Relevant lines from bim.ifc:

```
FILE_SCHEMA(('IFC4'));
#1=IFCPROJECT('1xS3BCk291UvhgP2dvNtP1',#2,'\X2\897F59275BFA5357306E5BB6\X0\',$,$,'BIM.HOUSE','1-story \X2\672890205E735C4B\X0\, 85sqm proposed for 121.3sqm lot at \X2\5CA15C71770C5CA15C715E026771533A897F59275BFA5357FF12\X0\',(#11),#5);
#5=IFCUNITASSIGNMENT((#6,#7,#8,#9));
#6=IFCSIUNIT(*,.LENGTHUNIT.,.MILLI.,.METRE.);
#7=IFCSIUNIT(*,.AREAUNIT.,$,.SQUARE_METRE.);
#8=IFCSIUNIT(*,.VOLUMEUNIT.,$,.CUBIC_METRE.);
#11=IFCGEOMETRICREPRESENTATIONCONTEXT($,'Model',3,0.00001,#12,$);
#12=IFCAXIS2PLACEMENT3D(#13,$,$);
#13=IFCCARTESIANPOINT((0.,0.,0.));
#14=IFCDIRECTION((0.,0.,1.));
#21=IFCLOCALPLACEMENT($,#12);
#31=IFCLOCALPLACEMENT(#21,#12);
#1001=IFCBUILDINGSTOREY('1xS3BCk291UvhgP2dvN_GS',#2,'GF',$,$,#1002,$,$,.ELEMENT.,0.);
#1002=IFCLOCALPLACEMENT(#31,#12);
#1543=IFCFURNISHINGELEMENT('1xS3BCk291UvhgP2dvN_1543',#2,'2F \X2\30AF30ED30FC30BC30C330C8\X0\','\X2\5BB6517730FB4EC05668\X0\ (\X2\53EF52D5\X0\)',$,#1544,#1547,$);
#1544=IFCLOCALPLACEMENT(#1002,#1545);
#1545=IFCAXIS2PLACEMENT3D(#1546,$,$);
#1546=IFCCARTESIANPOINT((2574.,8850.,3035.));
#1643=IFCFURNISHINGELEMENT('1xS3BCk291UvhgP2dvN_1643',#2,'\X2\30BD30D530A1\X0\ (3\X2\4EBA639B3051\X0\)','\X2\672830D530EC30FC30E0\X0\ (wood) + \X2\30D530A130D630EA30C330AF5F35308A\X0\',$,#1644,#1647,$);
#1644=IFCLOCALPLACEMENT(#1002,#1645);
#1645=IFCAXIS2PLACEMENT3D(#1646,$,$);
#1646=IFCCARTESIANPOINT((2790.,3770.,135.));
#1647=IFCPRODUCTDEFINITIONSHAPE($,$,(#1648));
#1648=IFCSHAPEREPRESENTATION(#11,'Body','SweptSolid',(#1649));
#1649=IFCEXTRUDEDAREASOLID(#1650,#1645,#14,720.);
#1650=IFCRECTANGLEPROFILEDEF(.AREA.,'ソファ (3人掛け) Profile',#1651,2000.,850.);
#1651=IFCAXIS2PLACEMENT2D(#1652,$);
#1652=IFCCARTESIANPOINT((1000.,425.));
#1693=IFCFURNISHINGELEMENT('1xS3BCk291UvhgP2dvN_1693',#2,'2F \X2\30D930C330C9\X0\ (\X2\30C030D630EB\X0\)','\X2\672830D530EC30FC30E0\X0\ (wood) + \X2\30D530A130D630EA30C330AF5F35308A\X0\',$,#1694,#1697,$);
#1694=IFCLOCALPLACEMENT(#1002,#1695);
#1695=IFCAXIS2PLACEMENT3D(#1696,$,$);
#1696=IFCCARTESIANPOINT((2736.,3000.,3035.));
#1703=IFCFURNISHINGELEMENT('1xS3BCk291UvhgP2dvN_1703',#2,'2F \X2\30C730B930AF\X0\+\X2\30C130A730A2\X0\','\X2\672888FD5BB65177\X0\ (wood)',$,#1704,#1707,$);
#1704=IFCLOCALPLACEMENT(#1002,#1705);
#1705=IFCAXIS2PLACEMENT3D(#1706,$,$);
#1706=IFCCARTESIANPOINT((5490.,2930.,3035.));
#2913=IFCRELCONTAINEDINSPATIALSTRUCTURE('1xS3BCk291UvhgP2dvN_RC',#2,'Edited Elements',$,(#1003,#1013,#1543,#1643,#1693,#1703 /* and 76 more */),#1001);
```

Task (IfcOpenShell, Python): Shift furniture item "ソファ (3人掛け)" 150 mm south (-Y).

```python
import ifcopenshell
import ifcopenshell.api.geometry
import ifcopenshell.util.placement
import ifcopenshell.util.unit

model = ifcopenshell.open("bim.ifc")
unit_scale = ifcopenshell.util.unit.calculate_unit_scale(model)

item = model.by_guid("1xS3BCk291UvhgP2dvN_1643")
matrix = ifcopenshell.util.placement.get_local_placement(item.ObjectPlacement)
matrix[1, 3] -= 0.15 / unit_scale
ifcopenshell.api.geometry.edit_object_placement(model, product=item, matrix=matrix, is_si=False)

print(ifcopenshell.util.placement.get_local_placement(item.ObjectPlacement).round(3) + 0.0)

model.write("bim_updated.ifc")
```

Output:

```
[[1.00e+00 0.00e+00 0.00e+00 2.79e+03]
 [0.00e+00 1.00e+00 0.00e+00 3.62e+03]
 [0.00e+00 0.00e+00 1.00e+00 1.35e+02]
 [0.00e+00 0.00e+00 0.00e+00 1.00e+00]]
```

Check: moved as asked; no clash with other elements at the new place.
